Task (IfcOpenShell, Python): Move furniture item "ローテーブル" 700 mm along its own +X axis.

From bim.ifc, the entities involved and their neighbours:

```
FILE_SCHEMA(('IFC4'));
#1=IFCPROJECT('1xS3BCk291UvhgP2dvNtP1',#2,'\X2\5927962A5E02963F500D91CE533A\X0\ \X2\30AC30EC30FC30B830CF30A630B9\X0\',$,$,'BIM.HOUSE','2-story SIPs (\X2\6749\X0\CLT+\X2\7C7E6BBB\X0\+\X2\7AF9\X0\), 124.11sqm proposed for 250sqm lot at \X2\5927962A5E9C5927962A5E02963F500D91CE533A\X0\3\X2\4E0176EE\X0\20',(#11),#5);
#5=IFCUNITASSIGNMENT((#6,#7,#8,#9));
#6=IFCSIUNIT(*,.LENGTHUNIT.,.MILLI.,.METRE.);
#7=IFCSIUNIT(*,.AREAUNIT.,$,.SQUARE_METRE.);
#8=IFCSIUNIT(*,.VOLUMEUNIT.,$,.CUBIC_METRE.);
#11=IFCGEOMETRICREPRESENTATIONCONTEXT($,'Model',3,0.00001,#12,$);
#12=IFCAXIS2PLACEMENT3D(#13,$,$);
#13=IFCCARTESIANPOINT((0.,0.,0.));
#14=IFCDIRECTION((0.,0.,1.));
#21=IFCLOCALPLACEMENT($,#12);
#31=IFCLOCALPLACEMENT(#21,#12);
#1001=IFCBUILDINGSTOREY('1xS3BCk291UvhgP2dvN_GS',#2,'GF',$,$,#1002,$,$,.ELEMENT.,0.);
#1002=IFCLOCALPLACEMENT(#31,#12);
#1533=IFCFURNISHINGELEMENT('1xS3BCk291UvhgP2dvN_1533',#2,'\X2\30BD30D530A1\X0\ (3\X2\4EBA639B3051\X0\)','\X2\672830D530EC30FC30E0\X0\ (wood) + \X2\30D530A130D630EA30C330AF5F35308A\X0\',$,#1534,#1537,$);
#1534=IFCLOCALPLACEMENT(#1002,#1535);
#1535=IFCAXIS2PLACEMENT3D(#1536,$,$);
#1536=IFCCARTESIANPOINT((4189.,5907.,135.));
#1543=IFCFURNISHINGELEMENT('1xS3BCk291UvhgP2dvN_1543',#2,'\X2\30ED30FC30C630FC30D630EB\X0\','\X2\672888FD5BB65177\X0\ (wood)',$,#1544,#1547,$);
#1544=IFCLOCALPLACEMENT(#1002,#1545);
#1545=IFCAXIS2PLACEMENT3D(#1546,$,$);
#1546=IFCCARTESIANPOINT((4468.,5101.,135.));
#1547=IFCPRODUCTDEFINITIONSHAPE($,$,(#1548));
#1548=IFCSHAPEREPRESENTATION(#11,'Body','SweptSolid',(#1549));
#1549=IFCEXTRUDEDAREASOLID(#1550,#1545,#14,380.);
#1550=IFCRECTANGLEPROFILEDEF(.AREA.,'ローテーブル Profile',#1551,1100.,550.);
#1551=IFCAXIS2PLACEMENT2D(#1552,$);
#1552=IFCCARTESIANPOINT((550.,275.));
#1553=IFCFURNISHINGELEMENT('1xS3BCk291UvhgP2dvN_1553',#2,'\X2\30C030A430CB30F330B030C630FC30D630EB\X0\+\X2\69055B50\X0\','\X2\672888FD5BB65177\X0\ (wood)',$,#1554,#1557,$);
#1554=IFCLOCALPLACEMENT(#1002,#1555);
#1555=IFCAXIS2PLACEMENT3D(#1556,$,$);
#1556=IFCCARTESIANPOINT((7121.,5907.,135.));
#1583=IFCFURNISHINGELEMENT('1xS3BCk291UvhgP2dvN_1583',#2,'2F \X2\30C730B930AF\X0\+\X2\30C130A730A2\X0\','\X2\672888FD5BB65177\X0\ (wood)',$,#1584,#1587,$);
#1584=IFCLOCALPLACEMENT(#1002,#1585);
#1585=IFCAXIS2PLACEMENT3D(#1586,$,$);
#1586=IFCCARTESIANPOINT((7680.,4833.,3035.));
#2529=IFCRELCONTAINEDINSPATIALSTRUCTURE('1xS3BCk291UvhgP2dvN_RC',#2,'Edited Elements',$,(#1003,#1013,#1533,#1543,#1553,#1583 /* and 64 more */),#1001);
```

```python
import ifcopenshell
import ifcopenshell.api.geometry
import ifcopenshell.util.placement

model = ifcopenshell.open("bim.ifc")

item = model.by_guid("1xS3BCk291UvhgP2dvN_1543")
matrix = ifcopenshell.util.placement.get_local_placement(item.ObjectPlacement)
matrix[:3, 3] += matrix[:3, 0] * 700.0
ifcopenshell.api.geometry.edit_object_placement(model, product=item, matrix=matrix, is_si=False)

print(ifcopenshell.util.placement.get_local_placement(item.ObjectPlacement).round(3) + 0.0)

model.write("bim_updated.ifc")
```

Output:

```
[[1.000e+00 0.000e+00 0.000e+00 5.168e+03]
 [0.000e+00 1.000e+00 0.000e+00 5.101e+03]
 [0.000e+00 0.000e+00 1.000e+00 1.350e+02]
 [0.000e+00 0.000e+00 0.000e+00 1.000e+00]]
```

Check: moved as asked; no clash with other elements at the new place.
